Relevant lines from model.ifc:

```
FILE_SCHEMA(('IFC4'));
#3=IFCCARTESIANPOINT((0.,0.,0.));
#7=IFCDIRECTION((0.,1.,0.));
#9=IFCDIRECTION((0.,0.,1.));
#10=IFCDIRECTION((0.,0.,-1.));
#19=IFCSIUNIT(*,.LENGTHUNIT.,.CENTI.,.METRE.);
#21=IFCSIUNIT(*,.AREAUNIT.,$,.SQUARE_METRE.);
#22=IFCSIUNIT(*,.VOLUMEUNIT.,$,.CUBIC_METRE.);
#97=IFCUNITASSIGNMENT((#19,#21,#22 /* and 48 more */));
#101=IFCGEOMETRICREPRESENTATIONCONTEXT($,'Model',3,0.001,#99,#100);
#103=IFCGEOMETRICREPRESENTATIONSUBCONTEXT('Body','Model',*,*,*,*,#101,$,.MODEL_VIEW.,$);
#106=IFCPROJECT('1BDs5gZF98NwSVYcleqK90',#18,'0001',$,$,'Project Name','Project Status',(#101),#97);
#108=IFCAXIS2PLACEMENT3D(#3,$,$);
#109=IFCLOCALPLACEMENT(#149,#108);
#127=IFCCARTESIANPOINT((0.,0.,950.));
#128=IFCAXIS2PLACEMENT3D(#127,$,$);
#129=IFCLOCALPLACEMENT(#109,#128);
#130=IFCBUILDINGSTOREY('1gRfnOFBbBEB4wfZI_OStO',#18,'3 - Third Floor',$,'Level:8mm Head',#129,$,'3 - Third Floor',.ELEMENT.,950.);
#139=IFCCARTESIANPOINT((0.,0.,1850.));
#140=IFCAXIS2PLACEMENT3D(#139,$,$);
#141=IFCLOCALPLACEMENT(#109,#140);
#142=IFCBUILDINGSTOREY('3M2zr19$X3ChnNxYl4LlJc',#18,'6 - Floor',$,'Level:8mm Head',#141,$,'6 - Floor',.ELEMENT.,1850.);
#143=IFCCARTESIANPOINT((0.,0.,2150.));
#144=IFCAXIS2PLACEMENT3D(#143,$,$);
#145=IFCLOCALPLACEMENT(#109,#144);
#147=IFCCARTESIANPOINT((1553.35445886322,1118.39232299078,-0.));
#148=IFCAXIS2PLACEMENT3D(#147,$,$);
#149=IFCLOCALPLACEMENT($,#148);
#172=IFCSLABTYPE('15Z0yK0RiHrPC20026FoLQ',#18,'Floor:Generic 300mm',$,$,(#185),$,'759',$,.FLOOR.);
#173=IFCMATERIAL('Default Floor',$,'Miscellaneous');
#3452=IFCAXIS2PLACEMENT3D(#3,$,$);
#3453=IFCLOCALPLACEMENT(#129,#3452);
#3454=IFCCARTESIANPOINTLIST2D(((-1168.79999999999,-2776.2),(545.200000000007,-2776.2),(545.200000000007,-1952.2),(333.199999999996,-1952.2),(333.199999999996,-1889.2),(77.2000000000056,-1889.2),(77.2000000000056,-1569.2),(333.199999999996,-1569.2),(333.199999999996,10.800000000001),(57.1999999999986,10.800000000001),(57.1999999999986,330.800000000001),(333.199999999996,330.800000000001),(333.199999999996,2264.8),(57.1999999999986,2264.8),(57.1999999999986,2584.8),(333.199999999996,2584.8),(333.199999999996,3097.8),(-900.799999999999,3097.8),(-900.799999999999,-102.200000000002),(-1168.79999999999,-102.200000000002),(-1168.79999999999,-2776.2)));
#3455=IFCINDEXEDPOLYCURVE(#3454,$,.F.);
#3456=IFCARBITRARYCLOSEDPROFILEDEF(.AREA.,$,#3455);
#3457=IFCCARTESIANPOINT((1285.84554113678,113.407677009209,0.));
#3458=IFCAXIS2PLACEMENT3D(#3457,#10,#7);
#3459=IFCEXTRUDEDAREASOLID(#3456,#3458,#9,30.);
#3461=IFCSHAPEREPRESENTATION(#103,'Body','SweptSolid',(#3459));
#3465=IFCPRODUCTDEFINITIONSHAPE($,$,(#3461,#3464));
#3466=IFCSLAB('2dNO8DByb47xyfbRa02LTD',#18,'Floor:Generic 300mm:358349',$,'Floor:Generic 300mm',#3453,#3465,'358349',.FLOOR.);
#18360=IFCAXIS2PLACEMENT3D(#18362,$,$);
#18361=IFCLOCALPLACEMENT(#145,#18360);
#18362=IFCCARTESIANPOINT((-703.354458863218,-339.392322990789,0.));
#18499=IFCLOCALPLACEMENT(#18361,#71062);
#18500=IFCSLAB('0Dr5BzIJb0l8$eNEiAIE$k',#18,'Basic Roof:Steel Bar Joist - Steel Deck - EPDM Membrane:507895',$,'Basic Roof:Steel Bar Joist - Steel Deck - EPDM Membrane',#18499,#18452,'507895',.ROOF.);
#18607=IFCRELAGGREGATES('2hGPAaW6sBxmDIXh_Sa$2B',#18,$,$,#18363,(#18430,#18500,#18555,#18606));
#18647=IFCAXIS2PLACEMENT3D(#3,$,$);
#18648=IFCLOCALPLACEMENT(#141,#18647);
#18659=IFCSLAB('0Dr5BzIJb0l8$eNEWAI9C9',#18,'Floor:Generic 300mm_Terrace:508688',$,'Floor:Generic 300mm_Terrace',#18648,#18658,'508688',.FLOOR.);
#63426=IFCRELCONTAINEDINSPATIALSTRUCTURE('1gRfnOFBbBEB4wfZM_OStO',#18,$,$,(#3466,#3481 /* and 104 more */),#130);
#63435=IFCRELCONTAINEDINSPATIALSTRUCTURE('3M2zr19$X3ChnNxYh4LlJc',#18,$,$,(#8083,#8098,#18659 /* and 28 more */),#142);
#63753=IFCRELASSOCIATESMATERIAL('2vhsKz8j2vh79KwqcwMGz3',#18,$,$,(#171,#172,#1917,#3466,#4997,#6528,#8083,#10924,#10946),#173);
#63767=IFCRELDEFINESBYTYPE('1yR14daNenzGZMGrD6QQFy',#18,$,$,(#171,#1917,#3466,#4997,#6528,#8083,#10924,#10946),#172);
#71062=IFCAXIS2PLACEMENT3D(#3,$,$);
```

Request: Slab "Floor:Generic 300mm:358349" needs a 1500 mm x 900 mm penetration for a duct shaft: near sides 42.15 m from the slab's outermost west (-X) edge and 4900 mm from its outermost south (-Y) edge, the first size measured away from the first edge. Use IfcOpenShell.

```python
import numpy as np
import ifcopenshell
import ifcopenshell.api.feature
import ifcopenshell.api.geometry
import ifcopenshell.api.root
import ifcopenshell.geom
import ifcopenshell.util.placement
import ifcopenshell.util.representation
import ifcopenshell.util.shape
import ifcopenshell.util.unit

model = ifcopenshell.open("model.ifc")
unit_scale = ifcopenshell.util.unit.calculate_unit_scale(model)
settings = ifcopenshell.geom.settings()


def volume(element):
    """Net volume in cubic metres, openings subtracted."""
    shape = ifcopenshell.geom.create_shape(settings, element)
    return ifcopenshell.util.shape.get_volume(shape.geometry)


slab = model.by_guid("2dNO8DByb47xyfbRa02LTD")
before = volume(slab)

# Extent in the slab's own axes, in metres. The edges named are its -X and -Y sides.
slab_shape = ifcopenshell.geom.create_shape(settings, slab)
vertices = ifcopenshell.util.shape.get_vertices(slab_shape.geometry)
x_min, y_min, bottom = vertices.min(axis=0)
top = vertices[:, 2].max()

opening = ifcopenshell.api.root.create_entity(model, ifc_class="IfcOpeningElement", name="Duct shaft opening", predefined_type="OPENING")
context = ifcopenshell.util.representation.get_context(model, "Model", "Body", "MODEL_VIEW")
width, depth = 1.5, 0.9
outline = [(0.0, 0.0), (width, 0.0), (width, depth), (0.0, depth), (0.0, 0.0)]
# Overshoot both faces by 50 mm so the cut is clean.
shape = ifcopenshell.api.geometry.add_slab_representation(
    model, context=context, depth=top - bottom + 0.1, polyline=outline
)
ifcopenshell.api.geometry.assign_representation(model, product=opening, representation=shape)

matrix = ifcopenshell.util.placement.get_local_placement(slab.ObjectPlacement)
matrix[:, 3] = matrix @ np.append(np.array([x_min + 42.15, y_min + 4.9, bottom - 0.05]) / unit_scale, 1.0)
ifcopenshell.api.geometry.edit_object_placement(model, product=opening, matrix=matrix, is_si=False)
ifcopenshell.api.feature.add_feature(model, feature=opening, element=slab)

after = volume(slab)

print(f"slab volume {before:.3f} -> {after:.3f} m3")

model.write("model-out.ifc")
```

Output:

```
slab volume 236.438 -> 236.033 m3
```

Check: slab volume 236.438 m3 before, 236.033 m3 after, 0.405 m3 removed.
